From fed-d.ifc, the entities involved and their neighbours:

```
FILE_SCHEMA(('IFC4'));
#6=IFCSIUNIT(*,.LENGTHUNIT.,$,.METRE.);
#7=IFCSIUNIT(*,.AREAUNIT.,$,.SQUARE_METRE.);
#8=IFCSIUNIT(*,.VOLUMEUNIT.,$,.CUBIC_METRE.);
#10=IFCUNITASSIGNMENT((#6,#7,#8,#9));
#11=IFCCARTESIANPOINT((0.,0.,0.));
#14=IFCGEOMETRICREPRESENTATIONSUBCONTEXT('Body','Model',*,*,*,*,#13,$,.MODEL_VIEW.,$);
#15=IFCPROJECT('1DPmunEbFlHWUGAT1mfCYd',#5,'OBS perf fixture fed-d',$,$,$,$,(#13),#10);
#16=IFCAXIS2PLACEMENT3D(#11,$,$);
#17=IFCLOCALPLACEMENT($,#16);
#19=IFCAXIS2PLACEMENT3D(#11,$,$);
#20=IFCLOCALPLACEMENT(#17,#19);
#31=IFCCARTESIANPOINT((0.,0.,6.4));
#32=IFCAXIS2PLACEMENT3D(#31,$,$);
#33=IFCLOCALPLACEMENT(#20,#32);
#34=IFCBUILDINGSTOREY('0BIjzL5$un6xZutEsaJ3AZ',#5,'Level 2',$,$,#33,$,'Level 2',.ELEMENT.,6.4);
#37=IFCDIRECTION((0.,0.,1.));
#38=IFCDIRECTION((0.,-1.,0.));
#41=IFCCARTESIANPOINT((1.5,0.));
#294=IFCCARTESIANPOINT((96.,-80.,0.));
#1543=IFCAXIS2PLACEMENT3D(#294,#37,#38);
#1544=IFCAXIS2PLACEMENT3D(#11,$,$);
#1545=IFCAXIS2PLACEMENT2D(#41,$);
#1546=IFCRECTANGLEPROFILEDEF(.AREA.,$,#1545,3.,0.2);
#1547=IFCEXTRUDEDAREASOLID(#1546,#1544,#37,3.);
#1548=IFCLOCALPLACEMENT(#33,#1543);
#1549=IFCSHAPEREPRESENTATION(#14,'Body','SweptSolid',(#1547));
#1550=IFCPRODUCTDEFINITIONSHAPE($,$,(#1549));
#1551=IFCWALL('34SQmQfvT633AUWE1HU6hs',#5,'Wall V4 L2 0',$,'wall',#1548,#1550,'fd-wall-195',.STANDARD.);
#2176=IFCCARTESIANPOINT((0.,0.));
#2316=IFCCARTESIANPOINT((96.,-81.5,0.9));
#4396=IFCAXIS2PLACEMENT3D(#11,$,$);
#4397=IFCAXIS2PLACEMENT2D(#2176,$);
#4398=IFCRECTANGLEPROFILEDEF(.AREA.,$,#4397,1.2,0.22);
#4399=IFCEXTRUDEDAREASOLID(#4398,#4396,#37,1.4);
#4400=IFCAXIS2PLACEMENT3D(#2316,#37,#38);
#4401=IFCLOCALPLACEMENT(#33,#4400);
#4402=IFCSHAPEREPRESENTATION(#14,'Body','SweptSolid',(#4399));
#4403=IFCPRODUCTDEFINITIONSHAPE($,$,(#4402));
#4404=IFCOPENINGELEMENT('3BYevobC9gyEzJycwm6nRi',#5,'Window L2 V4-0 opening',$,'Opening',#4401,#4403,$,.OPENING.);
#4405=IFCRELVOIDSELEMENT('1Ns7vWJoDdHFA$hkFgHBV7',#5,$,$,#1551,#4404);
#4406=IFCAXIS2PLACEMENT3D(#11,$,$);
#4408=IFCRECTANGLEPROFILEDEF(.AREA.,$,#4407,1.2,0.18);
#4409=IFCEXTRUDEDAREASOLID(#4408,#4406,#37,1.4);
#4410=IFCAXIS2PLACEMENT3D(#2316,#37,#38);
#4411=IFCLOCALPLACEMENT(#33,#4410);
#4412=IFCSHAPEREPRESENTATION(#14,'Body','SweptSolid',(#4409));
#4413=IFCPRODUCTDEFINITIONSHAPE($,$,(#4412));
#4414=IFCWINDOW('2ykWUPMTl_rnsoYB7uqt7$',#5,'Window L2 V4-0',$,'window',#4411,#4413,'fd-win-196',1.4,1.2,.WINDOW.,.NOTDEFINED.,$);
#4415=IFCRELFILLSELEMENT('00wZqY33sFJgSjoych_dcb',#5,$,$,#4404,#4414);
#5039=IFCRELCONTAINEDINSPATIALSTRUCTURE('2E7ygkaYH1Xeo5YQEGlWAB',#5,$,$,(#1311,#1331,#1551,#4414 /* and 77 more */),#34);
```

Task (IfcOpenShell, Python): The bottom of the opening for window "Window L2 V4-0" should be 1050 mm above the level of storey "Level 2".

```python
import numpy as np
import ifcopenshell
import ifcopenshell.api.geometry
import ifcopenshell.geom
import ifcopenshell.util.element
import ifcopenshell.util.placement
import ifcopenshell.util.shape
import ifcopenshell.util.unit

model = ifcopenshell.open("fed-d.ifc")
unit_scale = ifcopenshell.util.unit.calculate_unit_scale(model)

window = model.by_id(4414)
opening = window.FillsVoids[0].RelatingOpeningElement
storey = ifcopenshell.util.element.get_container(window, ifc_class="IfcBuildingStorey")
level = ifcopenshell.util.placement.get_local_placement(storey.ObjectPlacement)[2, 3]

# The opening's origin need not be at the sill, so measure its lowest point.
shape = ifcopenshell.geom.create_shape(ifcopenshell.geom.settings(), opening)
bottom = ifcopenshell.util.shape.get_shape_bottom_elevation(shape, shape.geometry) / unit_scale
dz = level + 1.05 / unit_scale - bottom

shift = np.array([0.0, 0.0, dz])
# The window is not placed relative to its opening, so move both.
for product in (opening, window):
    matrix = ifcopenshell.util.placement.get_local_placement(product.ObjectPlacement)
    matrix[:3, 3] += shift
    ifcopenshell.api.geometry.edit_object_placement(model, product=product, matrix=matrix, is_si=False)

print(f"moved by {dz * unit_scale:+.3f} m")

model.write("fed-d_rev.ifc")
```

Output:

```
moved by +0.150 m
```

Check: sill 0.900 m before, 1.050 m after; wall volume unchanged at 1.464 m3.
